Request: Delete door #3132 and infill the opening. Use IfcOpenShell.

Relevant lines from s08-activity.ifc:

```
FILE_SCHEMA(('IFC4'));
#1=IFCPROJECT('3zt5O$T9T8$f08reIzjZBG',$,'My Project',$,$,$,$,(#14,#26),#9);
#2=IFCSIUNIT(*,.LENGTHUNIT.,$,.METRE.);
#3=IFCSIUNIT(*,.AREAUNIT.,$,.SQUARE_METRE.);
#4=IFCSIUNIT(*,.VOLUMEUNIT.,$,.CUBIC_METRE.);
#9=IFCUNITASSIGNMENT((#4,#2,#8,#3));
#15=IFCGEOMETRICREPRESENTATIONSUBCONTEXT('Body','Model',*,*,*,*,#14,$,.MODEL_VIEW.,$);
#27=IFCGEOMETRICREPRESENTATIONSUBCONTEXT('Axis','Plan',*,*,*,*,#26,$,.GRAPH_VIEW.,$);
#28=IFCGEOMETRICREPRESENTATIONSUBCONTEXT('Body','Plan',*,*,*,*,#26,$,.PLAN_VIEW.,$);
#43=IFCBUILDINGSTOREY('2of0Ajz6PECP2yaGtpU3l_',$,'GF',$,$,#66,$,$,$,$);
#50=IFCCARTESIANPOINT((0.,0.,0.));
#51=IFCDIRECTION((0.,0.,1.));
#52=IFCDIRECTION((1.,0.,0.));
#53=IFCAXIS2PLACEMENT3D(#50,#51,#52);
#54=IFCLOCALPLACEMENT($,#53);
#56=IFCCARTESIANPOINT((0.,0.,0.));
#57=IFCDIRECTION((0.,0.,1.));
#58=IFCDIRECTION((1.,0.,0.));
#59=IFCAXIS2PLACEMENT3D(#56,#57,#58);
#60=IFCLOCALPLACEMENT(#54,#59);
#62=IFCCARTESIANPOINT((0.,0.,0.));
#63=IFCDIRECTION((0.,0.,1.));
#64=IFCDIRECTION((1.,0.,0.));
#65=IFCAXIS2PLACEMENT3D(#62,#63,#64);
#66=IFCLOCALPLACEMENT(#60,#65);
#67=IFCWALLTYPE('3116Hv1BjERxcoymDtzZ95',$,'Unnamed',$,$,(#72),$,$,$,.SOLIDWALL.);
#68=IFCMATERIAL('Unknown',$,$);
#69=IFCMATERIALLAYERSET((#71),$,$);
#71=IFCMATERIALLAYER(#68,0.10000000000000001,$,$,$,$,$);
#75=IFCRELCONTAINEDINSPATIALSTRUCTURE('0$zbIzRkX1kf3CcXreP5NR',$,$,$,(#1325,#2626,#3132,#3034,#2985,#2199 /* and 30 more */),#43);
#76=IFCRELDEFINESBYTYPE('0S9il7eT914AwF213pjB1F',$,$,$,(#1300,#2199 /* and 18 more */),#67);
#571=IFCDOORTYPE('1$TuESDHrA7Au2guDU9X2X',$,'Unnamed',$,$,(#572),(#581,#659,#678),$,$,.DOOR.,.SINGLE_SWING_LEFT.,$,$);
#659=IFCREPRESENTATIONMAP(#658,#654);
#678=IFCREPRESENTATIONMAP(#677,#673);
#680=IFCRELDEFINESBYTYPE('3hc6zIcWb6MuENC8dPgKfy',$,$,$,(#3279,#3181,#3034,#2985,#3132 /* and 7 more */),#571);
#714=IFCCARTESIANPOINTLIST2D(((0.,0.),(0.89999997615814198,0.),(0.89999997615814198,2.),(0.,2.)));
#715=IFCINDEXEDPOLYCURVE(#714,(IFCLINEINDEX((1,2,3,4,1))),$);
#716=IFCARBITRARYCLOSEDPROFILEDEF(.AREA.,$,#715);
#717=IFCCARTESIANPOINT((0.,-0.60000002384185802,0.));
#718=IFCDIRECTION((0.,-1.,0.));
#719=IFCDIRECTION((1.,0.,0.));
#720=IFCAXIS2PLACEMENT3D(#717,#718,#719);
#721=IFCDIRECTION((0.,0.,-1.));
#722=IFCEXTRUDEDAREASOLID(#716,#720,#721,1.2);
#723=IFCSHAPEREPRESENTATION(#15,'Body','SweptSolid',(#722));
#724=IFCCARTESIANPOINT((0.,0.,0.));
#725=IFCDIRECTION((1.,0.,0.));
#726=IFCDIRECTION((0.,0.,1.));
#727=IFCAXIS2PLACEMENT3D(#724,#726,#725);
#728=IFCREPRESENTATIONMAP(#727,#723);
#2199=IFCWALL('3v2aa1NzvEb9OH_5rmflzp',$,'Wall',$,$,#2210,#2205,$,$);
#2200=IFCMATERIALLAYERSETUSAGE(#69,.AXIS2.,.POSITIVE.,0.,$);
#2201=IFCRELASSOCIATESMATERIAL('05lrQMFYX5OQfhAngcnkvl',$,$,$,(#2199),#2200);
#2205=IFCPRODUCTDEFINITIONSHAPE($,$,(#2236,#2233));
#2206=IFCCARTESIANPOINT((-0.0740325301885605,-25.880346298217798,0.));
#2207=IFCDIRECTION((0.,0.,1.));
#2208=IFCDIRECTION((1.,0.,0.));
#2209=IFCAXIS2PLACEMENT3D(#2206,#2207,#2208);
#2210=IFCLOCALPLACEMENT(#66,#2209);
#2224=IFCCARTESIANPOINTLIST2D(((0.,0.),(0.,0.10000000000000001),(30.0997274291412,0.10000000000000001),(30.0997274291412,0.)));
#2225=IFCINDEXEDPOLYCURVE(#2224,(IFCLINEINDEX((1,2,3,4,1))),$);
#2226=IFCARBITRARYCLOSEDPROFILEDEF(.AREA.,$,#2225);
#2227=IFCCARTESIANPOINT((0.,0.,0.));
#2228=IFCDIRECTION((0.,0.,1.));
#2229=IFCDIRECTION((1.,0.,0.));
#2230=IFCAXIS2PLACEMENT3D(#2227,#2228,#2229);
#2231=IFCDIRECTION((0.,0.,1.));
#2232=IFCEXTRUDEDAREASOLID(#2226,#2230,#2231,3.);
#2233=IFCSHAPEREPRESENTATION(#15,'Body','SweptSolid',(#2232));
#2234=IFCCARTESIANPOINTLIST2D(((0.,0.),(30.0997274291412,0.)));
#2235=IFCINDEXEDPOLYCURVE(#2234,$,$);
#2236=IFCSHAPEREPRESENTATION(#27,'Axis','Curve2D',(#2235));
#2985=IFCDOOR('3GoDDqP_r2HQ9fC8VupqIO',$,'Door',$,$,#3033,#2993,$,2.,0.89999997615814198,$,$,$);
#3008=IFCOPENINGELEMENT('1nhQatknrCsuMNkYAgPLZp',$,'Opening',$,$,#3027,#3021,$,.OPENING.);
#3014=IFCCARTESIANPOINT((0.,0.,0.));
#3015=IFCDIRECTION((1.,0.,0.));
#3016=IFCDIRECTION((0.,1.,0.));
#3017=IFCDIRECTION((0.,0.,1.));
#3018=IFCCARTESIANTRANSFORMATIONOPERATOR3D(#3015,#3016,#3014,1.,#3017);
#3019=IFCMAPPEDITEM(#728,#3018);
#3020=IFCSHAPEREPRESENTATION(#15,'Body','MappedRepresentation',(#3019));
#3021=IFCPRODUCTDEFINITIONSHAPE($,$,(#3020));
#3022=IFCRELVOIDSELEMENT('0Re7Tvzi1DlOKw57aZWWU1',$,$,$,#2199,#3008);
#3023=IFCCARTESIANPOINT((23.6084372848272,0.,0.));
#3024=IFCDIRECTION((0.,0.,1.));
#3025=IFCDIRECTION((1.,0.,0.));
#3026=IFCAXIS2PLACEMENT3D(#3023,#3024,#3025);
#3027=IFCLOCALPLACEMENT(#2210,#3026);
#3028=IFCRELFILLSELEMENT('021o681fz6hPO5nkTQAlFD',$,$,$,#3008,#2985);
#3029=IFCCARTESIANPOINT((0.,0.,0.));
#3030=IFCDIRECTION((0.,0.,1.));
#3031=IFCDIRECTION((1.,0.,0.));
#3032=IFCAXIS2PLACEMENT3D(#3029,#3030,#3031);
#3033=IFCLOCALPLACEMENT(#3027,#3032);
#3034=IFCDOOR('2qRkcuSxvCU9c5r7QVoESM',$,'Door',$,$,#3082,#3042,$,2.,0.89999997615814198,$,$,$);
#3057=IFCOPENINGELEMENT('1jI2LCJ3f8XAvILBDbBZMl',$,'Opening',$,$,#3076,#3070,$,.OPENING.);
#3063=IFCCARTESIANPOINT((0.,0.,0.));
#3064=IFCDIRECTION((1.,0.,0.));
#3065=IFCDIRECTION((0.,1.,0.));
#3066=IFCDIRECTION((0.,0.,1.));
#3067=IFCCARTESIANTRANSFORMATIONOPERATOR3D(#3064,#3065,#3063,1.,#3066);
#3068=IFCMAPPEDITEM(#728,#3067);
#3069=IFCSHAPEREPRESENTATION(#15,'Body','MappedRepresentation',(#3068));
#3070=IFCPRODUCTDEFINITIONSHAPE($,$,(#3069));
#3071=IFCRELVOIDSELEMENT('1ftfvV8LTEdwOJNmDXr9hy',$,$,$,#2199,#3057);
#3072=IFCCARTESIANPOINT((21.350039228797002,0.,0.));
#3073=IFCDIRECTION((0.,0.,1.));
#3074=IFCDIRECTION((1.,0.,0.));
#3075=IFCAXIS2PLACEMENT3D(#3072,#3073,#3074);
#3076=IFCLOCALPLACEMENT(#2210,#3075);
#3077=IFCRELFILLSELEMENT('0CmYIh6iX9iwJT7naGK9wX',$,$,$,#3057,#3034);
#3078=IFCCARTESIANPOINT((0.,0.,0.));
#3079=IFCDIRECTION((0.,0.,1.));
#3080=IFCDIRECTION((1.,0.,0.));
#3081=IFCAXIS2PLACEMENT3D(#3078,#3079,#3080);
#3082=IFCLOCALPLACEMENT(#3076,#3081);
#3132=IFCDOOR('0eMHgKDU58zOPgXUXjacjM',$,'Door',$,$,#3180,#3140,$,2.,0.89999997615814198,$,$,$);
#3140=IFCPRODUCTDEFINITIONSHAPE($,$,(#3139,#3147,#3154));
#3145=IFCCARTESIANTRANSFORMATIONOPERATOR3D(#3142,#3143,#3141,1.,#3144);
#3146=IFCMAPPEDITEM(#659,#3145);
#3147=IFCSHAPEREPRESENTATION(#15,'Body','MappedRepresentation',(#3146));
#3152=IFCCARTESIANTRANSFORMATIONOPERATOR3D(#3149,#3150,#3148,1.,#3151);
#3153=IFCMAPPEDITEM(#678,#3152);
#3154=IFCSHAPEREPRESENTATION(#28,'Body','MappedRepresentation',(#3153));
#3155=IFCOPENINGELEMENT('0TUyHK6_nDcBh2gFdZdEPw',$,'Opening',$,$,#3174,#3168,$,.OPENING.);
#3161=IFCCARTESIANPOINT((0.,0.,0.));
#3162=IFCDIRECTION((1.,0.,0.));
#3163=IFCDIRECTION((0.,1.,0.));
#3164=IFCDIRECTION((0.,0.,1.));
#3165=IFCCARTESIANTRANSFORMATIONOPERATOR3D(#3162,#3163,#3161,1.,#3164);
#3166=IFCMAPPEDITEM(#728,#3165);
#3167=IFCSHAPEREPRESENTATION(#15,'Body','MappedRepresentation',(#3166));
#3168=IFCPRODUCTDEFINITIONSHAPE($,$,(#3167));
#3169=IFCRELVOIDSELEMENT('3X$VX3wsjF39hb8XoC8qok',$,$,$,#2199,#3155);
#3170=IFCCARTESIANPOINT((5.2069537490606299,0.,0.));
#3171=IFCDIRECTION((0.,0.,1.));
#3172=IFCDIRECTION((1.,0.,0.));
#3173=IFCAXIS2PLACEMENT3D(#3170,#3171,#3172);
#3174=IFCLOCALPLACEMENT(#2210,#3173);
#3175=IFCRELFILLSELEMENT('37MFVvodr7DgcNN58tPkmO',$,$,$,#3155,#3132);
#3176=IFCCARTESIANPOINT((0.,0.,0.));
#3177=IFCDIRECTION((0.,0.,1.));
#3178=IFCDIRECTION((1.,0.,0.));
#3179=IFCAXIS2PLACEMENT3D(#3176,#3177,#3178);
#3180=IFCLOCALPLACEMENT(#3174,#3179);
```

```python
import ifcopenshell
import ifcopenshell.api.feature
import ifcopenshell.api.root
import ifcopenshell.geom
import ifcopenshell.util.shape

model = ifcopenshell.open("s08-activity.ifc")
settings = ifcopenshell.geom.settings()


def volume(element):
    """Net volume in cubic metres, openings subtracted."""
    shape = ifcopenshell.geom.create_shape(settings, element)
    return ifcopenshell.util.shape.get_volume(shape.geometry)


door = model.by_guid("0eMHgKDU58zOPgXUXjacjM")
opening = door.FillsVoids[0].RelatingOpeningElement
wall = opening.VoidsElements[0].RelatingBuildingElement
before = volume(wall)

ifcopenshell.api.root.remove_product(model, product=door)
ifcopenshell.api.feature.remove_feature(model, feature=opening)

after = volume(wall)

print(f"wall volume {before:.3f} -> {after:.3f} m3")

model.write("s08-activity_edited.ifc")
```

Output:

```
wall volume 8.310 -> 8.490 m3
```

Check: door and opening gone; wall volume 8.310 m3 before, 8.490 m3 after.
